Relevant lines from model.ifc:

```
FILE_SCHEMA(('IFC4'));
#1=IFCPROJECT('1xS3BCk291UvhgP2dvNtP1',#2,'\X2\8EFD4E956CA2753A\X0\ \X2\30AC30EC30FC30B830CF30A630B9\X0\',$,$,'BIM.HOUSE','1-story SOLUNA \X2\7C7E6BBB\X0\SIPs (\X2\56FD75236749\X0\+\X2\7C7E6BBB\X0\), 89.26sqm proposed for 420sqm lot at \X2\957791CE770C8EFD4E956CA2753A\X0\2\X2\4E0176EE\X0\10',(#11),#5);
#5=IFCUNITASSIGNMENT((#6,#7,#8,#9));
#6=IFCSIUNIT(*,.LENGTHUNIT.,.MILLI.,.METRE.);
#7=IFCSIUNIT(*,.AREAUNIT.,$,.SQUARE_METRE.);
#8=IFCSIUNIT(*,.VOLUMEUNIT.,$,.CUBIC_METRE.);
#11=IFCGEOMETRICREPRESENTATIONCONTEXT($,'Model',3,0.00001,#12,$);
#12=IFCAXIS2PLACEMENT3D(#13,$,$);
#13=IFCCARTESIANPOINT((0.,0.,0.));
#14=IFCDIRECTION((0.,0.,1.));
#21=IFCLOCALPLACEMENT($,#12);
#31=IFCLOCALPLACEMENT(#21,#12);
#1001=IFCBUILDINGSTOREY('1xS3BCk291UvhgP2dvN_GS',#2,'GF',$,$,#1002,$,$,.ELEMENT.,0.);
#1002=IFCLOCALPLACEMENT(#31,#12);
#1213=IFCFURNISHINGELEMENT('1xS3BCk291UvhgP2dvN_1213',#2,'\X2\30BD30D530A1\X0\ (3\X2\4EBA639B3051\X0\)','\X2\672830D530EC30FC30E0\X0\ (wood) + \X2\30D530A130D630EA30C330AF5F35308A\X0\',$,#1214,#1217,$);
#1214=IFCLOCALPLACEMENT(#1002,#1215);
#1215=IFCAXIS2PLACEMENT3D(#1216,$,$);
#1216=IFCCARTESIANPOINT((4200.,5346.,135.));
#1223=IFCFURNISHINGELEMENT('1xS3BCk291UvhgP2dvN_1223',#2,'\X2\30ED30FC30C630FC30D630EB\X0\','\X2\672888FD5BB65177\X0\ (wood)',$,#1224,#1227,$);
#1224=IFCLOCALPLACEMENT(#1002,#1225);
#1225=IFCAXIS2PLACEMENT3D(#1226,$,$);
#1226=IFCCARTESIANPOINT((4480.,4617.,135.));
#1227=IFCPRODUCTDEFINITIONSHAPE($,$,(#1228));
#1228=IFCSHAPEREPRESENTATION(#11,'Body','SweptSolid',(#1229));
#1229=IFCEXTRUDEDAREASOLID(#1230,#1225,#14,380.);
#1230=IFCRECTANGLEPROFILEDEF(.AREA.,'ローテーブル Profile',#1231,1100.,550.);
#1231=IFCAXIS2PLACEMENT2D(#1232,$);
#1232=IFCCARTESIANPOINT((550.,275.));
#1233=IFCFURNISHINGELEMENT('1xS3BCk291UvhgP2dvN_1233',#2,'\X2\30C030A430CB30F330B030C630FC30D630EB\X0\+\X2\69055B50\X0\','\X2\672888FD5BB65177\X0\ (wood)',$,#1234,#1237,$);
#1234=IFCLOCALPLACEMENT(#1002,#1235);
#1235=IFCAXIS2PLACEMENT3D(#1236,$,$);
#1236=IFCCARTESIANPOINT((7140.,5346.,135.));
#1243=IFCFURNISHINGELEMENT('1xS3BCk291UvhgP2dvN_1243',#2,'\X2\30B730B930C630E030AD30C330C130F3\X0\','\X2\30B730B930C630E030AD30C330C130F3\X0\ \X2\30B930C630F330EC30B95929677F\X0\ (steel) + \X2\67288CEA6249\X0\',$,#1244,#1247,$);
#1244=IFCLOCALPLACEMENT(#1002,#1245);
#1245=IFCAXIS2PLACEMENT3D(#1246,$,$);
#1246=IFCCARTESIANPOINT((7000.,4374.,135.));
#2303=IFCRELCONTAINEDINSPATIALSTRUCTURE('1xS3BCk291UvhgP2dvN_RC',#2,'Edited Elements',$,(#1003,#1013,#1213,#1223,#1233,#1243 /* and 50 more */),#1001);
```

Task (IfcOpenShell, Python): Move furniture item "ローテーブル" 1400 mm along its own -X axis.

```python
import ifcopenshell
import ifcopenshell.api.geometry
import ifcopenshell.util.placement
import ifcopenshell.util.unit

model = ifcopenshell.open("model.ifc")
unit_scale = ifcopenshell.util.unit.calculate_unit_scale(model)

item = model.by_id(1223)
matrix = ifcopenshell.util.placement.get_local_placement(item.ObjectPlacement)
matrix[:3, 3] -= matrix[:3, 0] * 1.4 / unit_scale
ifcopenshell.api.geometry.edit_object_placement(model, product=item, matrix=matrix, is_si=False)

print(ifcopenshell.util.placement.get_local_placement(item.ObjectPlacement).round(3) + 0.0)

model.write("model_edited.ifc")
```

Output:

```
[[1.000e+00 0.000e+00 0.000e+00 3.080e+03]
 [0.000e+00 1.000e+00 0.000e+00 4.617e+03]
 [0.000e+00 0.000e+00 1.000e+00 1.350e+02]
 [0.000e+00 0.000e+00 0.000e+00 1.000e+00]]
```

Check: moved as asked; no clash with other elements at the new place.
